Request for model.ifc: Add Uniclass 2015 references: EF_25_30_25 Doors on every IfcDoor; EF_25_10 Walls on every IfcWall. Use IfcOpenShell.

First a look at what the model holds.

```python
import ifcopenshell

model = ifcopenshell.open("model.ifc")
print(model.schema)
print("classifications:", [c.Name for c in model.by_type("IfcClassification")])
for ifc_class in ("IfcDoor", "IfcRoof", "IfcStair", "IfcWall", "IfcWindow"):
    print(ifc_class, len(model.by_type(ifc_class)))
```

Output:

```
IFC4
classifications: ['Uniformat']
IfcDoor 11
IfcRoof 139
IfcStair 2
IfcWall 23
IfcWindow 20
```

```python
import ifcopenshell
import ifcopenshell.api.classification

model = ifcopenshell.open("model.ifc")

system = ifcopenshell.api.classification.add_classification(model, classification="Uniclass 2015")

codes = {
    "IfcDoor": ("EF_25_30_25", "Doors"),
    "IfcWall": ("EF_25_10", "Walls"),
}
for ifc_class, (code, name) in codes.items():
    products = model.by_type(ifc_class)
    ifcopenshell.api.classification.add_reference(
        model, products=products, classification=system, identification=code, name=name
    )
    print(code, len(products))

model.write("model-out.ifc")
```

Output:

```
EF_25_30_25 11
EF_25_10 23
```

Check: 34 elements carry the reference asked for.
